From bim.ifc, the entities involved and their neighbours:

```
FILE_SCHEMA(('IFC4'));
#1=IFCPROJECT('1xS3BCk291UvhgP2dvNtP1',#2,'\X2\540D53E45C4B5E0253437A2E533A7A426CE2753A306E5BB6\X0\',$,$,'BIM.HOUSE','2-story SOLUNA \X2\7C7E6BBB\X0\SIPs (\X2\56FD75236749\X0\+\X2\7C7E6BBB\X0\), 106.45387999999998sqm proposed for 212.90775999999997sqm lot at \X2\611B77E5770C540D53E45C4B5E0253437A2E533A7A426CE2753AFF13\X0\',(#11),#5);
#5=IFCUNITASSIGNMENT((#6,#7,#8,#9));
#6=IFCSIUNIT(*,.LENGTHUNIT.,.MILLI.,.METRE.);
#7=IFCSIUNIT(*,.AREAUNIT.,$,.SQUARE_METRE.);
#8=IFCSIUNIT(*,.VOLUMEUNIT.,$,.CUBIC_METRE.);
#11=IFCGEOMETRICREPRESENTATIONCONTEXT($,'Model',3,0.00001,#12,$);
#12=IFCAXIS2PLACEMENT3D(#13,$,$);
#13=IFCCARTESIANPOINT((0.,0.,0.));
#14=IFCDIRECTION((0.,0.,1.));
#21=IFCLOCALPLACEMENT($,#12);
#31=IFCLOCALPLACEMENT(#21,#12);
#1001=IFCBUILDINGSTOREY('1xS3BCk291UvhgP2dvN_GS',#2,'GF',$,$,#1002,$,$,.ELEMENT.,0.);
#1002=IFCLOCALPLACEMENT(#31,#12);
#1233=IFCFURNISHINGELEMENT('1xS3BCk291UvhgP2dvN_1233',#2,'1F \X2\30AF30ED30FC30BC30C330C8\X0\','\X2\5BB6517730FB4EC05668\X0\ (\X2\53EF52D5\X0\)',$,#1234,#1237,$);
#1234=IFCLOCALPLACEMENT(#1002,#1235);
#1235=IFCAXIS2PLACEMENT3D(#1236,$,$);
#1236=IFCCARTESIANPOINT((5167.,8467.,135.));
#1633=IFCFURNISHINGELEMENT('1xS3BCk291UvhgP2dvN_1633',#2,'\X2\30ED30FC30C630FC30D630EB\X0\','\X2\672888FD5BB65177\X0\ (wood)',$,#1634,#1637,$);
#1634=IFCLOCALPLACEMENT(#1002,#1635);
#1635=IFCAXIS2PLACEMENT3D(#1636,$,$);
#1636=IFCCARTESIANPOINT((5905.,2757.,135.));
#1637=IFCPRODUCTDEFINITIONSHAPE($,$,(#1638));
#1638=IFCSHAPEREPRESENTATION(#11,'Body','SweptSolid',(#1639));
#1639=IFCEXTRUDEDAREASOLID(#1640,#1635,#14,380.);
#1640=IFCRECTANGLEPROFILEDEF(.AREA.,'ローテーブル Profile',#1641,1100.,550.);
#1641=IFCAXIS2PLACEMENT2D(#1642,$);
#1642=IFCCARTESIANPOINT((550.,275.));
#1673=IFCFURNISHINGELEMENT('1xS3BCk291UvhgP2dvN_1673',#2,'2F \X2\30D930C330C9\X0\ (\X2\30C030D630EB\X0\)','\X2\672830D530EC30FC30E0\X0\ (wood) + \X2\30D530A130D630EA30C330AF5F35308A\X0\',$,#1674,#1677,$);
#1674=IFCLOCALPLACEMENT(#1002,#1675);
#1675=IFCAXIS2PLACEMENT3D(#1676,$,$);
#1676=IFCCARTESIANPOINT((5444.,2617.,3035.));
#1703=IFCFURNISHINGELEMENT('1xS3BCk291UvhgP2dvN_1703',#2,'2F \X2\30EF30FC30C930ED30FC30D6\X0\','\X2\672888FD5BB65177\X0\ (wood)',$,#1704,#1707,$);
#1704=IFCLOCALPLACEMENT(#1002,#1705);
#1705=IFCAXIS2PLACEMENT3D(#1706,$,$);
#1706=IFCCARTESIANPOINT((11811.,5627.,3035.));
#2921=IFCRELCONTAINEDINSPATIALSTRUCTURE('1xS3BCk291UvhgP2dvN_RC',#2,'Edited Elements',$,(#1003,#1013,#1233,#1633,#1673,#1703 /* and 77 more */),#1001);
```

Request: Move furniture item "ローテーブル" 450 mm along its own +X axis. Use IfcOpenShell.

```python
import ifcopenshell
import ifcopenshell.api.geometry
import ifcopenshell.util.placement

model = ifcopenshell.open("bim.ifc")

item = model.by_guid("1xS3BCk291UvhgP2dvN_1633")
matrix = ifcopenshell.util.placement.get_local_placement(item.ObjectPlacement)
matrix[:3, 3] += matrix[:3, 0] * 450.0
ifcopenshell.api.geometry.edit_object_placement(model, product=item, matrix=matrix, is_si=False)

print(ifcopenshell.util.placement.get_local_placement(item.ObjectPlacement).round(3) + 0.0)

model.write("bim_rev.ifc")
```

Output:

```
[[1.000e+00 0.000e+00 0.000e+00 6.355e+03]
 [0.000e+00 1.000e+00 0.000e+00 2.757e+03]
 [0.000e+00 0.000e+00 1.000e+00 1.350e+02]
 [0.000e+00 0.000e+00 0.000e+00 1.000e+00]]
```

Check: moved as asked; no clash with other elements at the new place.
